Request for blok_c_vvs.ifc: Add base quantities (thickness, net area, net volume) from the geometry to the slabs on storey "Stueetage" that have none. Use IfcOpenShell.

First a look at what the model holds.

```python
import ifcopenshell
import ifcopenshell.util.element
import ifcopenshell.util.unit

model = ifcopenshell.open("blok_c_vvs.ifc")
print(model.schema)
for unit_type in ("LENGTHUNIT", "AREAUNIT", "VOLUMEUNIT"):
    print(unit_type, ifcopenshell.util.unit.calculate_unit_scale(model, unit_type))
storey = next(s for s in model.by_type("IfcBuildingStorey") if s.Name == "Stueetage")
slabs = [e for e in ifcopenshell.util.element.get_decomposition(storey) if e.is_a("IfcSlab")]
for e in sorted(slabs, key=lambda e: e.id()):
    print(e.id(), e.is_a(), e.Name, list(ifcopenshell.util.element.get_psets(e, qtos_only=True)), sep=" | ")
```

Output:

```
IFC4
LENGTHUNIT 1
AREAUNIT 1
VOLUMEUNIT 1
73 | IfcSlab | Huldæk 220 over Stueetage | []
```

```python
import ifcopenshell
import ifcopenshell.api.pset
import ifcopenshell.geom
import ifcopenshell.util.element
import ifcopenshell.util.shape
import ifcopenshell.util.unit

model = ifcopenshell.open("blok_c_vvs.ifc")
unit_scale = ifcopenshell.util.unit.calculate_unit_scale(model)
area_scale = ifcopenshell.util.unit.calculate_unit_scale(model, "AREAUNIT")
volume_scale = ifcopenshell.util.unit.calculate_unit_scale(model, "VOLUMEUNIT")
settings = ifcopenshell.geom.settings()

storey = next(s for s in model.by_type("IfcBuildingStorey") if s.Name == "Stueetage")
slabs = [e for e in ifcopenshell.util.element.get_decomposition(storey) if e.is_a("IfcSlab")]

for e in sorted(slabs, key=lambda e: e.id()):
    if ifcopenshell.util.element.get_psets(e, qtos_only=True, should_inherit=False):
        continue
    # Geometry comes back in metres, in the element's own axes.
    shape = ifcopenshell.geom.create_shape(settings, e)
    values = {
        "Width": ifcopenshell.util.shape.get_z(shape.geometry) / unit_scale,
        "NetArea": ifcopenshell.util.shape.get_footprint_area(shape.geometry) / area_scale,
        "NetVolume": ifcopenshell.util.shape.get_volume(shape.geometry) / volume_scale,
    }
    qto = ifcopenshell.api.pset.add_qto(model, product=e, name="Qto_SlabBaseQuantities")
    ifcopenshell.api.pset.edit_qto(model, qto=qto, properties=values)
    print(e.id(), {k: round(v, 3) for k, v in values.items()})

model.write("blok_c_vvs_updated.ifc")
```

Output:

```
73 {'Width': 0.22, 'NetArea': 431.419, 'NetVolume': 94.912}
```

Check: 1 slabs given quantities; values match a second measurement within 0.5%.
